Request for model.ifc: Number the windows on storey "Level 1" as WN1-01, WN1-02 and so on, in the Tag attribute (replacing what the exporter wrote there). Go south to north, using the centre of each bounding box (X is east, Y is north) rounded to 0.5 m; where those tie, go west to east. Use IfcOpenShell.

First a look at what the model holds.

```python
import ifcopenshell
import ifcopenshell.util.element
import ifcopenshell.util.placement

model = ifcopenshell.open("model.ifc")
print(model.schema)
storey = next(s for s in model.by_type("IfcBuildingStorey") if s.Name == "Level 1")
windows = [e for e in ifcopenshell.util.element.get_decomposition(storey) if e.is_a("IfcWindow")]
for e in sorted(windows, key=lambda e: e.id()):
    origin = ifcopenshell.util.placement.get_local_placement(e.ObjectPlacement)[:3, 3]
    print(e.id(), e.Tag, e.Name, origin.round(2) + 0.0, sep=" | ")
```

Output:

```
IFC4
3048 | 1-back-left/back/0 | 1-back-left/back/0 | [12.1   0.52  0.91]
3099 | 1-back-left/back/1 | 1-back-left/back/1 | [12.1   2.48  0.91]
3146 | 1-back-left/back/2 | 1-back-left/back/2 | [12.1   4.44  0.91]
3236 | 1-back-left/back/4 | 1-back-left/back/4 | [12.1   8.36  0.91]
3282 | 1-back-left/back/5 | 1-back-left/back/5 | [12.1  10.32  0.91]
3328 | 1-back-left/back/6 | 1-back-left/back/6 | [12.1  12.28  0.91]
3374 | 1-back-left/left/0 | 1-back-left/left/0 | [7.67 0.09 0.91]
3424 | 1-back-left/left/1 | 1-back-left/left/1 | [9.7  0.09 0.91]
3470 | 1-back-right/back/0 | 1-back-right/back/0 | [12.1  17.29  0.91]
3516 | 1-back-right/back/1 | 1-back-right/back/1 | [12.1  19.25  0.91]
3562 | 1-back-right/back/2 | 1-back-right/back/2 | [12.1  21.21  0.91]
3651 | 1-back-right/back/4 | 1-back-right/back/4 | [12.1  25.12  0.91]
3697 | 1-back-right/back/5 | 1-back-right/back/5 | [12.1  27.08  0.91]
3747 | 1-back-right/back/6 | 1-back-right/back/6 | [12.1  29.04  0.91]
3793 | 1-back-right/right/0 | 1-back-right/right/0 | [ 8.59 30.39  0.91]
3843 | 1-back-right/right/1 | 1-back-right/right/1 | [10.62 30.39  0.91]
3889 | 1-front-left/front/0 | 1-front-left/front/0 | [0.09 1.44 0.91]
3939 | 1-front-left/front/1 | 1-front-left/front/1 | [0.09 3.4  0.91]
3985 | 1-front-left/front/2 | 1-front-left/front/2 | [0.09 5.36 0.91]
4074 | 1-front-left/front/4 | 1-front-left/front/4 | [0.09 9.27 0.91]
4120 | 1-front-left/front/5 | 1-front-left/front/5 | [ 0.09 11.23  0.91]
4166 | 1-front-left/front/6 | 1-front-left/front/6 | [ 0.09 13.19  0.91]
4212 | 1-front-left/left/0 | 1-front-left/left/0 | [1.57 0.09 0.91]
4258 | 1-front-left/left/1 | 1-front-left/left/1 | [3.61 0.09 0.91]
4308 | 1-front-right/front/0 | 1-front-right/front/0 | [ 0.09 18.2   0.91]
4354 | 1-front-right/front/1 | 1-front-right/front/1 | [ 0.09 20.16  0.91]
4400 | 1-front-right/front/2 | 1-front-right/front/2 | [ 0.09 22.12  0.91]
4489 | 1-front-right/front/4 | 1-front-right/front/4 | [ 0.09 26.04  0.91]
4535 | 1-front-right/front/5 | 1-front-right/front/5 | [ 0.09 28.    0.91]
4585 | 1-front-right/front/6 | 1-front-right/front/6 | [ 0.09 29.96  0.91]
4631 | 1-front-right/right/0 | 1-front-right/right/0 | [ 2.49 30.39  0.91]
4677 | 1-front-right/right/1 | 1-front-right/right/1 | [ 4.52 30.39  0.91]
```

```python
import ifcopenshell
import ifcopenshell.geom
import ifcopenshell.util.element
import ifcopenshell.util.shape

model = ifcopenshell.open("model.ifc")
settings = ifcopenshell.geom.settings()
settings.set("use-world-coords", True)


def centre(element):
    shape = ifcopenshell.geom.create_shape(settings, element)
    return ifcopenshell.util.shape.get_bbox_centroid(shape.geometry)


storey = next(s for s in model.by_type("IfcBuildingStorey") if s.Name == "Level 1")
windows = [e for e in ifcopenshell.util.element.get_decomposition(storey) if e.is_a("IfcWindow")]

# Insertion points can sit at a corner or the storey origin, so sort by the geometry (in metres).
centres = {e: centre(e) for e in windows}
windows.sort(key=lambda e: (round(centres[e][1] / 0.5), centres[e][0]))

for i, e in enumerate(windows, start=1):
    number = f"WN1-{i:02d}"
    e.Tag = number
    print(e.id(), number)

model.write("model_rev.ifc")
```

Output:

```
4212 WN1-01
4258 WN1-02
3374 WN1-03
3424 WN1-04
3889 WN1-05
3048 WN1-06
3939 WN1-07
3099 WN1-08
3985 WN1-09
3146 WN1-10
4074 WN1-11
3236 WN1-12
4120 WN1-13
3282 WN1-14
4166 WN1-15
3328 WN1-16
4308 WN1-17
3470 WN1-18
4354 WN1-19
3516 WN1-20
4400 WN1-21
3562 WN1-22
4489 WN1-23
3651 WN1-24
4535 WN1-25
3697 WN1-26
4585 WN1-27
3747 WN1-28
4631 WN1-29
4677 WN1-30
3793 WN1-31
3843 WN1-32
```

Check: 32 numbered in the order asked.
